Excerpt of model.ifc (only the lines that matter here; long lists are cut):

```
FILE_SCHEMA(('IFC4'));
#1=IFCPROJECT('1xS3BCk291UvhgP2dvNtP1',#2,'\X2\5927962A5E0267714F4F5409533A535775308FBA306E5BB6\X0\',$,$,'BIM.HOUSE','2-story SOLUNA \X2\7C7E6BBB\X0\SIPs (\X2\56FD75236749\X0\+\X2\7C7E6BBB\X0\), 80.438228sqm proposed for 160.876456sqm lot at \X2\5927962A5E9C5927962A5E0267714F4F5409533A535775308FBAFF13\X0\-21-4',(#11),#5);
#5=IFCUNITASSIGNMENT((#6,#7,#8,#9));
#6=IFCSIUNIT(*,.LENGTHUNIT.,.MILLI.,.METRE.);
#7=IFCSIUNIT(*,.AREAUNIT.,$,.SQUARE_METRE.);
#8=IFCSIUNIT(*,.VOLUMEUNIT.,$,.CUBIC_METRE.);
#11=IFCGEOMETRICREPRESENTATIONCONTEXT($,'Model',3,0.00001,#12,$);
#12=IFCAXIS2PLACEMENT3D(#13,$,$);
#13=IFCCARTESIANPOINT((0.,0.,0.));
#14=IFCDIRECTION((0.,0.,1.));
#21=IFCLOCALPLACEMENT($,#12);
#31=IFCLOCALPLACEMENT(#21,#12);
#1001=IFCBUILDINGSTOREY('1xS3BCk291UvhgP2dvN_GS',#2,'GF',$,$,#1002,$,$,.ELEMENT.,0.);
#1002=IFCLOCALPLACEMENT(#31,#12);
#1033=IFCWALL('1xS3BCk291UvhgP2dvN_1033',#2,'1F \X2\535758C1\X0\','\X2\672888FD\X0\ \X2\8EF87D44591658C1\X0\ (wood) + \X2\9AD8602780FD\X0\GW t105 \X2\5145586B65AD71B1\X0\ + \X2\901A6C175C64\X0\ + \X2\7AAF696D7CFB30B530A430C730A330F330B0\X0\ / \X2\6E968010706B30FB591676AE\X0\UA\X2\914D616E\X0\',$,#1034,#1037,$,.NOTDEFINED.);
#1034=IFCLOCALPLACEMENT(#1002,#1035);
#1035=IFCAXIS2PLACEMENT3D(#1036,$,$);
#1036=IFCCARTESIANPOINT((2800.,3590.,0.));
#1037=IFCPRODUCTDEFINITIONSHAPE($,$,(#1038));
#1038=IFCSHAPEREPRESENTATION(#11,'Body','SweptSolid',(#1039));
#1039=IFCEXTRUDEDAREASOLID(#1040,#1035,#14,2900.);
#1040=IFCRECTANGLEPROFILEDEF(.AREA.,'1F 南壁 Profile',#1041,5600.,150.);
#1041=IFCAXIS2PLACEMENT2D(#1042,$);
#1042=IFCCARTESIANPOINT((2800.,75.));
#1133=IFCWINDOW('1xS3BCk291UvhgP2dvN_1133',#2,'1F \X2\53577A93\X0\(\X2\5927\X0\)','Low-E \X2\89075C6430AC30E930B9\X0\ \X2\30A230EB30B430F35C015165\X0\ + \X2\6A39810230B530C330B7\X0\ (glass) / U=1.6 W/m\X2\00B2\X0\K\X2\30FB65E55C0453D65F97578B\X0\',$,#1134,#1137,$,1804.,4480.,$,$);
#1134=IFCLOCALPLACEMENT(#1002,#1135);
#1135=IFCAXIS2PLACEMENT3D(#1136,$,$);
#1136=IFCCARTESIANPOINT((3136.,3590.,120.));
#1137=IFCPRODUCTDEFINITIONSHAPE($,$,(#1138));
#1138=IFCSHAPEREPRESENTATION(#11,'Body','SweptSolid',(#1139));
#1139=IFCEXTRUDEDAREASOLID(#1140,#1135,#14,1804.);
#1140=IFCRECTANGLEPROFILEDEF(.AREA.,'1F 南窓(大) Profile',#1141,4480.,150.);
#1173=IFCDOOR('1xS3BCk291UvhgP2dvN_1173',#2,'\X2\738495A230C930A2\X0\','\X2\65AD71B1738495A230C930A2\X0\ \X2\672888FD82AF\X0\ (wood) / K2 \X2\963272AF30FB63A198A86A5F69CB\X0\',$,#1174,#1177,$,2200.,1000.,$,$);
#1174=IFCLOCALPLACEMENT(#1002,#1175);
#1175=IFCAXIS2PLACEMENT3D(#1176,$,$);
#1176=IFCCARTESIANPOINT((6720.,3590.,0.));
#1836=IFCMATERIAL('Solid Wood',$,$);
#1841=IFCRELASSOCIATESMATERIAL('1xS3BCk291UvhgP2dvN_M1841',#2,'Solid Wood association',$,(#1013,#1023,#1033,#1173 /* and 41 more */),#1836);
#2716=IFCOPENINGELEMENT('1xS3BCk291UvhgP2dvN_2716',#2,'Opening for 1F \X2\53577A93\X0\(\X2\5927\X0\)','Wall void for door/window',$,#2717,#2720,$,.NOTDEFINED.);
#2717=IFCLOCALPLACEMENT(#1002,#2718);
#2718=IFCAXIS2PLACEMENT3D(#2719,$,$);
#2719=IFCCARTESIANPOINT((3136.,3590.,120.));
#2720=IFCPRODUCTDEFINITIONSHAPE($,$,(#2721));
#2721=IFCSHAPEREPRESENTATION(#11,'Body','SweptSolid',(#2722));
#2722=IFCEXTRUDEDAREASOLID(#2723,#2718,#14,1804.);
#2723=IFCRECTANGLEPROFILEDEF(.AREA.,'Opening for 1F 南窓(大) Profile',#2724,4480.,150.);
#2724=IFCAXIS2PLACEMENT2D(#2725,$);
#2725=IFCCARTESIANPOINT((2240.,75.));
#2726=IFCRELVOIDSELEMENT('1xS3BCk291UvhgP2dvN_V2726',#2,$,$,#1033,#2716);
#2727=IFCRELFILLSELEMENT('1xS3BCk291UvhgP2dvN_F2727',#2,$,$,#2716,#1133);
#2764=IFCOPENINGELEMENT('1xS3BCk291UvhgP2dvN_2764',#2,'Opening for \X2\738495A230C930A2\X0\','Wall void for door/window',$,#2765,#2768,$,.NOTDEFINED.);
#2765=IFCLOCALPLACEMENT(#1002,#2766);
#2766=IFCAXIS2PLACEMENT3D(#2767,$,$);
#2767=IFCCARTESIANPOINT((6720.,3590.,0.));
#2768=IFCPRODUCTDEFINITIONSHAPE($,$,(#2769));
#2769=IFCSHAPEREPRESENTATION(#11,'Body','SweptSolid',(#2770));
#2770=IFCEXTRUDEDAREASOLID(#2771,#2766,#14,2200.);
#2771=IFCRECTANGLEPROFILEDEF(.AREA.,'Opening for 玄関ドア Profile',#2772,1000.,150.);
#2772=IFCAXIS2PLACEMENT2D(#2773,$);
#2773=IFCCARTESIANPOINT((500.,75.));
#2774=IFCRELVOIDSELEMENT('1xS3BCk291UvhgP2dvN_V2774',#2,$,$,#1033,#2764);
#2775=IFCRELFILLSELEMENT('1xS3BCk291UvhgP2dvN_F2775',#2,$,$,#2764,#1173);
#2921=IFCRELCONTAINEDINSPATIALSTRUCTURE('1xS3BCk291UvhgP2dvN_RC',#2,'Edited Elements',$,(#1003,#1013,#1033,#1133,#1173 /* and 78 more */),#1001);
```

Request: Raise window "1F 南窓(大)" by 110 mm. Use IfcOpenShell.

```python
import numpy as np
import ifcopenshell
import ifcopenshell.api.geometry
import ifcopenshell.util.placement
import ifcopenshell.util.unit

model = ifcopenshell.open("model.ifc")
unit_scale = ifcopenshell.util.unit.calculate_unit_scale(model)

window = model.by_guid("1xS3BCk291UvhgP2dvN_1133")
opening = window.FillsVoids[0].RelatingOpeningElement
dz = 0.11 / unit_scale

shift = np.array([0.0, 0.0, dz])
# The window is not placed relative to its opening, so move both.
for product in (opening, window):
    matrix = ifcopenshell.util.placement.get_local_placement(product.ObjectPlacement)
    matrix[:3, 3] += shift
    ifcopenshell.api.geometry.edit_object_placement(model, product=product, matrix=matrix, is_si=False)

print(f"moved by {dz * unit_scale:+.3f} m")

model.write("model_v2.ifc")
```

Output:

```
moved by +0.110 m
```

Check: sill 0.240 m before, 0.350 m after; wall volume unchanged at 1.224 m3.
